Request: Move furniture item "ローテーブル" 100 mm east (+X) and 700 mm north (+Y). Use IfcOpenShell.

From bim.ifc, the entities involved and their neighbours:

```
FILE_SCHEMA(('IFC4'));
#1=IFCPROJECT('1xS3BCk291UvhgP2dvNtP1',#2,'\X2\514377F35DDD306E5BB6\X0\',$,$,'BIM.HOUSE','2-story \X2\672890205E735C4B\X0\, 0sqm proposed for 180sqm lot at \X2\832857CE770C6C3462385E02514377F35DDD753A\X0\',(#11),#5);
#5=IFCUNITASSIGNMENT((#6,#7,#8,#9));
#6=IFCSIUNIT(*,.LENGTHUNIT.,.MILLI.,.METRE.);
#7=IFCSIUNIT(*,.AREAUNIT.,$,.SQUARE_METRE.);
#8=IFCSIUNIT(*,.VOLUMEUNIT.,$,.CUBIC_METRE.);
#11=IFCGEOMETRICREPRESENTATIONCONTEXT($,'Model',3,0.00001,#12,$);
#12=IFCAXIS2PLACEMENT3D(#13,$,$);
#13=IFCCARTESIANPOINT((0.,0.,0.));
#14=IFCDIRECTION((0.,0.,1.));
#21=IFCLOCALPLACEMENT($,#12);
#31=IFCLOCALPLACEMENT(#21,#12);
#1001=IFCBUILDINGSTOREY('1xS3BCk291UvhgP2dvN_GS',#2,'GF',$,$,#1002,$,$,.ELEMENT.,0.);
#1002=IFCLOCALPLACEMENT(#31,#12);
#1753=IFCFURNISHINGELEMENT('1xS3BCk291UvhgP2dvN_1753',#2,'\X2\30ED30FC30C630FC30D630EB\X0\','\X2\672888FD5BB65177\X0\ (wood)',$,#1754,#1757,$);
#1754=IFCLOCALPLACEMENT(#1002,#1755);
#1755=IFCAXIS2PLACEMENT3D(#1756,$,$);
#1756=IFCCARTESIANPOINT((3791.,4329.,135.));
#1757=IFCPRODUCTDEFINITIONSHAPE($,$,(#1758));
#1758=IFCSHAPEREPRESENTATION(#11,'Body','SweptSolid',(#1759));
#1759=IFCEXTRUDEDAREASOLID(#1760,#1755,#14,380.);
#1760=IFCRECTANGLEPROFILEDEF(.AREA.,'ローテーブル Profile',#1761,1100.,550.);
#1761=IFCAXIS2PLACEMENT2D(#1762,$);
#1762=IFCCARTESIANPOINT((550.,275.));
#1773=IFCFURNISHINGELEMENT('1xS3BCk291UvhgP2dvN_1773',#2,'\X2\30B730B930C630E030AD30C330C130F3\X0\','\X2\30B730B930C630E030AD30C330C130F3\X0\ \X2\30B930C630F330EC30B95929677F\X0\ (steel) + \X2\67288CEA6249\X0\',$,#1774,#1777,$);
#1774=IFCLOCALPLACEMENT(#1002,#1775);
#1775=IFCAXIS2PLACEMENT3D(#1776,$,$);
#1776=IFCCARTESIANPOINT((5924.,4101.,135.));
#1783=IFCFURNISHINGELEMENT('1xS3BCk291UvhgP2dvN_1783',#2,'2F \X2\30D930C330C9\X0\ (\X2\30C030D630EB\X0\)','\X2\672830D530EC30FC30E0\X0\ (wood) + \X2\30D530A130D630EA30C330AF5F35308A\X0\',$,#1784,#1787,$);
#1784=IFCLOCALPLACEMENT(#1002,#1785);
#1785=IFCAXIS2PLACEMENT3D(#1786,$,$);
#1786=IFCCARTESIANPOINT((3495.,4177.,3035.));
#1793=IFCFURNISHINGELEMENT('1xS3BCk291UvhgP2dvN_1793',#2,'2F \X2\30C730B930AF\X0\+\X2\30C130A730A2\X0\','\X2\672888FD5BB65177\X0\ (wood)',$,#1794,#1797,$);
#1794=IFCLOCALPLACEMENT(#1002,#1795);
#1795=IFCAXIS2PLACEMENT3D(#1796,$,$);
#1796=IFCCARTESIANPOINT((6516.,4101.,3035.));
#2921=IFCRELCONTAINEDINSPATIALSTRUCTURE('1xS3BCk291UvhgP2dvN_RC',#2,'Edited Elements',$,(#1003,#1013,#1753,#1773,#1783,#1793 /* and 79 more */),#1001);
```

```python
import ifcopenshell
import ifcopenshell.api.geometry
import ifcopenshell.util.placement

model = ifcopenshell.open("bim.ifc")

item = model.by_guid("1xS3BCk291UvhgP2dvN_1753")
matrix = ifcopenshell.util.placement.get_local_placement(item.ObjectPlacement)
matrix[0, 3] += 100.0
matrix[1, 3] += 700.0
ifcopenshell.api.geometry.edit_object_placement(model, product=item, matrix=matrix, is_si=False)

print(ifcopenshell.util.placement.get_local_placement(item.ObjectPlacement).round(3) + 0.0)

model.write("bim_updated.ifc")
```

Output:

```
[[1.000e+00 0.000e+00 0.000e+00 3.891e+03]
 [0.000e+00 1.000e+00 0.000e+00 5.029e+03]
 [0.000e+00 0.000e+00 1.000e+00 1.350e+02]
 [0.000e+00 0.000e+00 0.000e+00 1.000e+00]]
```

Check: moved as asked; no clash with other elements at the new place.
